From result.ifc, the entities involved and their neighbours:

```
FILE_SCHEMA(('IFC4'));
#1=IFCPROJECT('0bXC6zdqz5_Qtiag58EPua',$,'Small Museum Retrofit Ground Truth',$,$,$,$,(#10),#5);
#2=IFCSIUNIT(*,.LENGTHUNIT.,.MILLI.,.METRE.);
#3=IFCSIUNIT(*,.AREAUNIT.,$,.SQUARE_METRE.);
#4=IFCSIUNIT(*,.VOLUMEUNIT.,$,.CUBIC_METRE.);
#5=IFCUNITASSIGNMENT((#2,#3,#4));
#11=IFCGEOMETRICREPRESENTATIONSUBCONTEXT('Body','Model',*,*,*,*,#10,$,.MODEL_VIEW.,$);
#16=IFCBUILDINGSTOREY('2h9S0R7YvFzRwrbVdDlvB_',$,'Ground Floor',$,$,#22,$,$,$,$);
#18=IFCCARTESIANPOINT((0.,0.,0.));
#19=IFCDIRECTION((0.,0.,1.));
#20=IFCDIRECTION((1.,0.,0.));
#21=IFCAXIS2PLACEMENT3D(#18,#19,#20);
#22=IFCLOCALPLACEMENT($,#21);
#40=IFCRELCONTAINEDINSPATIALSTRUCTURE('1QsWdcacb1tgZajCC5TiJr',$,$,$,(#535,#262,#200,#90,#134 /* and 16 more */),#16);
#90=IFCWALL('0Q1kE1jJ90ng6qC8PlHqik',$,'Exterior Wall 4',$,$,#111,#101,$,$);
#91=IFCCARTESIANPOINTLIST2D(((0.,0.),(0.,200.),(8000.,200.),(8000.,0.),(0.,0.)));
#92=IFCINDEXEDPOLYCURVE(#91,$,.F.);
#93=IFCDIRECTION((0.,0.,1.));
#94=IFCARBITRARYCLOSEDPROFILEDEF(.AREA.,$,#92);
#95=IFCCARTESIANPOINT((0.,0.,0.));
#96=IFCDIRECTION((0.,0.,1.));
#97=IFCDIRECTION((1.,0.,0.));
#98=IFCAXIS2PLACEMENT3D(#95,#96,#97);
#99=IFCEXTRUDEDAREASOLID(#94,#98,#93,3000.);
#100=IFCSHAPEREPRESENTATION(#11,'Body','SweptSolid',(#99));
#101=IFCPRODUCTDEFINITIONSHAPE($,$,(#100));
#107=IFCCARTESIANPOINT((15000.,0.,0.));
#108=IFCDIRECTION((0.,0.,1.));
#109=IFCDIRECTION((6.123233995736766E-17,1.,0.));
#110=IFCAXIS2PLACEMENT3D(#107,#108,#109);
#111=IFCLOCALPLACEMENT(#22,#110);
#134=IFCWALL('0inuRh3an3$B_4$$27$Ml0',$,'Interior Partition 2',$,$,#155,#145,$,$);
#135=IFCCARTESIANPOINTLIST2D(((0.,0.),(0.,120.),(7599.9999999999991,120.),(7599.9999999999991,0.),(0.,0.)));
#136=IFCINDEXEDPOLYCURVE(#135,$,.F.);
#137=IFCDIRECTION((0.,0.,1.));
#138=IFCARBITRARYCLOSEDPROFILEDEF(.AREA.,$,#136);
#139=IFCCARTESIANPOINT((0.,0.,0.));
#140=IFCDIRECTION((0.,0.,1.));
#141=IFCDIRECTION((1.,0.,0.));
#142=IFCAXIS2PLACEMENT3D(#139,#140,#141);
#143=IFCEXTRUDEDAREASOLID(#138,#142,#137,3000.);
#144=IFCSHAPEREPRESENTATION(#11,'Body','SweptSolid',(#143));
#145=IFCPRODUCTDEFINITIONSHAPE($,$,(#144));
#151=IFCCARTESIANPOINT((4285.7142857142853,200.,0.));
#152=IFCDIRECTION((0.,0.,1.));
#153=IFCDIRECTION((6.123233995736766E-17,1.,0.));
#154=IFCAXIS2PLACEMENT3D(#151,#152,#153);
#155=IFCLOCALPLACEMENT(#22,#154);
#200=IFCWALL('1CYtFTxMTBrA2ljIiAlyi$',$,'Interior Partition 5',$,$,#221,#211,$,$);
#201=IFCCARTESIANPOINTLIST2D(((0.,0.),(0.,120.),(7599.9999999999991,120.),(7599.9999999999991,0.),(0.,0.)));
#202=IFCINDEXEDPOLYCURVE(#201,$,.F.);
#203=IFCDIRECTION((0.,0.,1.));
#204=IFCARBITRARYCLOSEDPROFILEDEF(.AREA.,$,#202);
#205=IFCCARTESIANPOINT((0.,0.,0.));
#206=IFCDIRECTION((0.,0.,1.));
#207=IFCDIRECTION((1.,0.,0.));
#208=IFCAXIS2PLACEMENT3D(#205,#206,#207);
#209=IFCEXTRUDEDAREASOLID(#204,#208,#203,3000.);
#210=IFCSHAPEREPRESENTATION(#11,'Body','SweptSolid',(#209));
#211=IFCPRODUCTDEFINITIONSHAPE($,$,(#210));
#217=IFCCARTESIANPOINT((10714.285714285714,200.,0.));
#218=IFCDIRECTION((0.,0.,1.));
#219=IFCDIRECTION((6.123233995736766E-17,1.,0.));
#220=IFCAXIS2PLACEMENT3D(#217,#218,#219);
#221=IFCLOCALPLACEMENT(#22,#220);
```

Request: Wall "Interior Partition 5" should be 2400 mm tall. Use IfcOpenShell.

```python
import ifcopenshell
import ifcopenshell.geom
import ifcopenshell.util.representation
import ifcopenshell.util.shape

model = ifcopenshell.open("result.ifc")
settings = ifcopenshell.geom.settings()


def volume(element):
    """Net volume in cubic metres, openings subtracted."""
    shape = ifcopenshell.geom.create_shape(settings, element)
    return ifcopenshell.util.shape.get_volume(shape.geometry)


wall = model.by_id(200)
before = volume(wall)

body = ifcopenshell.util.representation.get_representation(wall, "Model", "Body")
solid = body.Items[0]
old_height = solid.Depth
solid.Depth = 2400.0
after = volume(wall)

print(f"height {old_height:g} -> {solid.Depth:g}, volume {before:.3f} -> {after:.3f} m3")

model.write("result-out.ifc")
```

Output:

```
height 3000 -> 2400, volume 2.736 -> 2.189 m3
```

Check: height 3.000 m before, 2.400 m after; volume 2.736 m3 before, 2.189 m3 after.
